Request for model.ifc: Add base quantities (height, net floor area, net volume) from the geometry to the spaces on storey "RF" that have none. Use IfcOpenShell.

First a look at what the model holds.

```python
import ifcopenshell
import ifcopenshell.util.element
import ifcopenshell.util.unit

model = ifcopenshell.open("model.ifc")
print(model.schema)
for unit_type in ("LENGTHUNIT", "AREAUNIT", "VOLUMEUNIT"):
    print(unit_type, ifcopenshell.util.unit.calculate_unit_scale(model, unit_type))
storey = next(s for s in model.by_type("IfcBuildingStorey") if s.Name == "RF")
spaces = [e for e in ifcopenshell.util.element.get_decomposition(storey) if e.is_a("IfcSpace")]
for e in sorted(spaces, key=lambda e: e.id()):
    print(e.id(), e.is_a(), e.Name, list(ifcopenshell.util.element.get_psets(e, qtos_only=True)), sep=" | ")
```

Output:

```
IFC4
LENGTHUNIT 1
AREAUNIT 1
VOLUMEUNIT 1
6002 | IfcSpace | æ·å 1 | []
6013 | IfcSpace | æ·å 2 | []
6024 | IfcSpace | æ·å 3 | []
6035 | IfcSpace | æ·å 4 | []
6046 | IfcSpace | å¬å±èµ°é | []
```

```python
import ifcopenshell
import ifcopenshell.api.pset
import ifcopenshell.geom
import ifcopenshell.util.element
import ifcopenshell.util.shape
import ifcopenshell.util.unit

model = ifcopenshell.open("model.ifc")
unit_scale = ifcopenshell.util.unit.calculate_unit_scale(model)
area_scale = ifcopenshell.util.unit.calculate_unit_scale(model, "AREAUNIT")
volume_scale = ifcopenshell.util.unit.calculate_unit_scale(model, "VOLUMEUNIT")
settings = ifcopenshell.geom.settings()

storey = next(s for s in model.by_type("IfcBuildingStorey") if s.Name == "RF")
spaces = [e for e in ifcopenshell.util.element.get_decomposition(storey) if e.is_a("IfcSpace")]

for e in sorted(spaces, key=lambda e: e.id()):
    if ifcopenshell.util.element.get_psets(e, qtos_only=True, should_inherit=False):
        continue
    # Geometry comes back in metres, in the element's own axes.
    shape = ifcopenshell.geom.create_shape(settings, e)
    values = {
        "Height": ifcopenshell.util.shape.get_z(shape.geometry) / unit_scale,
        "NetFloorArea": ifcopenshell.util.shape.get_footprint_area(shape.geometry) / area_scale,
        "NetVolume": ifcopenshell.util.shape.get_volume(shape.geometry) / volume_scale,
    }
    qto = ifcopenshell.api.pset.add_qto(model, product=e, name="Qto_SpaceBaseQuantities")
    ifcopenshell.api.pset.edit_qto(model, qto=qto, properties=values)
    print(e.id(), {k: round(v, 3) for k, v in values.items()})

model.write("model_updated.ifc")
```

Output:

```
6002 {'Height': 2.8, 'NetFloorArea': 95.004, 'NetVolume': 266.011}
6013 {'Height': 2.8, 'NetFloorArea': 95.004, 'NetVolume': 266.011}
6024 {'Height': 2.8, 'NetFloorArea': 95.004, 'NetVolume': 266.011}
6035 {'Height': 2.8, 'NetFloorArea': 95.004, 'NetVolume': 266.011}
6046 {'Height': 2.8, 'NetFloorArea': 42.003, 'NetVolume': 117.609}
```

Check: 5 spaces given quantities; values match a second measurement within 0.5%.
